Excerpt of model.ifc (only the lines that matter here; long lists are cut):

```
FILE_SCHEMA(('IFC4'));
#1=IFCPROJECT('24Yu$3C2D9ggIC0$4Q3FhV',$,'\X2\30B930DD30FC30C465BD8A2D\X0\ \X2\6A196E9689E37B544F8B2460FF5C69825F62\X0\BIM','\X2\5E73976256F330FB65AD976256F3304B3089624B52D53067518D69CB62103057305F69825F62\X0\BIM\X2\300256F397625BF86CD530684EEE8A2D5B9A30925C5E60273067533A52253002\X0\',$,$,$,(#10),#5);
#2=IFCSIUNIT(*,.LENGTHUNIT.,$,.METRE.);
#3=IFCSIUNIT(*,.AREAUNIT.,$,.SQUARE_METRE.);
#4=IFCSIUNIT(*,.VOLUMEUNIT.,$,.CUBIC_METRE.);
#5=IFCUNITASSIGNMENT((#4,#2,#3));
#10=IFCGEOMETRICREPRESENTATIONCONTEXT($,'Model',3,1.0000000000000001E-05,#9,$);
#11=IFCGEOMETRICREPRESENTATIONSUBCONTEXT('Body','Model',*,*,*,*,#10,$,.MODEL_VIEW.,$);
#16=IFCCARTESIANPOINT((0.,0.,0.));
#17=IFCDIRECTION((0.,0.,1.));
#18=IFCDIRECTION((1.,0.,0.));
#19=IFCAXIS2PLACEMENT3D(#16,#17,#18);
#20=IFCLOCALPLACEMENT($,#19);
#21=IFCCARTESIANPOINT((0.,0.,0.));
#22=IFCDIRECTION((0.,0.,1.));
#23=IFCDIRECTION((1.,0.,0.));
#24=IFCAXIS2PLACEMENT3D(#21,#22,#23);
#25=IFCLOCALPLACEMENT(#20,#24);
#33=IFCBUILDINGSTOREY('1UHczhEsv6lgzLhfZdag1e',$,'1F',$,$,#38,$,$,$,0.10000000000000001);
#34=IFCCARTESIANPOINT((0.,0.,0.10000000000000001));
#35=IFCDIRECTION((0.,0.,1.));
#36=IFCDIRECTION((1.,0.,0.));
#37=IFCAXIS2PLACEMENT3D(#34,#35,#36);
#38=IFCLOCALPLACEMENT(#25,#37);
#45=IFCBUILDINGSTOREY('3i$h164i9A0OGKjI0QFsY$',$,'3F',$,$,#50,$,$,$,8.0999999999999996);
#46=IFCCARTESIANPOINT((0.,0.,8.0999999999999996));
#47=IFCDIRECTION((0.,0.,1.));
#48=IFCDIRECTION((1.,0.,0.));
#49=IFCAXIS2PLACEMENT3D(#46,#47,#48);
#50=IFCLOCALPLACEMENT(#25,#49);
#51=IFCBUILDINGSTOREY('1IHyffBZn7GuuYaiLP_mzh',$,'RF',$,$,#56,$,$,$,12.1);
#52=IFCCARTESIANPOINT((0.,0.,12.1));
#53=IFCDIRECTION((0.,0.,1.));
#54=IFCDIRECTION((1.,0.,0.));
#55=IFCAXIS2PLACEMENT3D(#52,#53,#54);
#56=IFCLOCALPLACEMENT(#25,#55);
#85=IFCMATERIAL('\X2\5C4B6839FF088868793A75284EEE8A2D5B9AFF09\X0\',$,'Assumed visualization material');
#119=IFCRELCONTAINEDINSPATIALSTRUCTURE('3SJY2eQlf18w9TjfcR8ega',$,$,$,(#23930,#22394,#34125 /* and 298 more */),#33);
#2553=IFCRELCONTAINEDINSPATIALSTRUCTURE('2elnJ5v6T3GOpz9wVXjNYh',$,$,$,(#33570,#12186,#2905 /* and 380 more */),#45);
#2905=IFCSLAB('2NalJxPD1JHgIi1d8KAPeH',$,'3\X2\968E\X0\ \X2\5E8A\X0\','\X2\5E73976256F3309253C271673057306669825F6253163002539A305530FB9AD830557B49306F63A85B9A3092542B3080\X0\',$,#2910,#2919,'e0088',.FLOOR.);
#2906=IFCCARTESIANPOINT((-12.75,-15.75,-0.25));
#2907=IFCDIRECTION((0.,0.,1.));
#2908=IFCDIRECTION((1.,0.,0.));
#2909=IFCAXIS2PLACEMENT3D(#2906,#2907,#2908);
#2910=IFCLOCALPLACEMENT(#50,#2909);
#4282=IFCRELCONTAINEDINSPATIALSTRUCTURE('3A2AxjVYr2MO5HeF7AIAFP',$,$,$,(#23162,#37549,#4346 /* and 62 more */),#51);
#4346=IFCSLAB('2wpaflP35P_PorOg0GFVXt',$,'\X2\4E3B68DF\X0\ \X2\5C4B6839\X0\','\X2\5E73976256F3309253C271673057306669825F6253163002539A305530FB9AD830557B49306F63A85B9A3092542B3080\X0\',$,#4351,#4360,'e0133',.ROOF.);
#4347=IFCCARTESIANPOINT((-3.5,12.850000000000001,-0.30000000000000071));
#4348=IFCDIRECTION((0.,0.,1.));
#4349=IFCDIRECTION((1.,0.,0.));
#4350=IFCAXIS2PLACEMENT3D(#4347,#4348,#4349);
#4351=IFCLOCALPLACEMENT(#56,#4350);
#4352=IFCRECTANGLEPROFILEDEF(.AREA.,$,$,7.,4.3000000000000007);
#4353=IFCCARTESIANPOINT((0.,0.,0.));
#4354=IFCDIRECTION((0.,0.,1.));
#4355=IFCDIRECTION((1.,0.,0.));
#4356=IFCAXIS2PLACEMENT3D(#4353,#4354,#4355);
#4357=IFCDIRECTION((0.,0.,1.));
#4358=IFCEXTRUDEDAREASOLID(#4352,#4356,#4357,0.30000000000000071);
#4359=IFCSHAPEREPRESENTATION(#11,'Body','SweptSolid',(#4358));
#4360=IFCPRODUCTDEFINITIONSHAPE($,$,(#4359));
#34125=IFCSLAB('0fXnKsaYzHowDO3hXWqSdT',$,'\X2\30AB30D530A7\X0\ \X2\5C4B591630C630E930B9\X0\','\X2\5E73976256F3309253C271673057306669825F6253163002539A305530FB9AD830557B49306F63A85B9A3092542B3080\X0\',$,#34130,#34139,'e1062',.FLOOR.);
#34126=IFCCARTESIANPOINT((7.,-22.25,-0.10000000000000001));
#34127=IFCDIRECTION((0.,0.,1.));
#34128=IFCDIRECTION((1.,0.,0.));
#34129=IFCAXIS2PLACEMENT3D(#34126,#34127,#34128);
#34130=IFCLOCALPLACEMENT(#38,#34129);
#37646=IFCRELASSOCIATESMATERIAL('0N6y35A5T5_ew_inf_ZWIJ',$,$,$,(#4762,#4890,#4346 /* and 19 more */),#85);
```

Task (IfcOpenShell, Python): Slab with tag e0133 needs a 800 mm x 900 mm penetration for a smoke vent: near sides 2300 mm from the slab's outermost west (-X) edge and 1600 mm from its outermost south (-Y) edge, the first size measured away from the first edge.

```python
import numpy as np
import ifcopenshell
import ifcopenshell.api.feature
import ifcopenshell.api.geometry
import ifcopenshell.api.root
import ifcopenshell.geom
import ifcopenshell.util.placement
import ifcopenshell.util.representation
import ifcopenshell.util.shape
import ifcopenshell.util.unit

model = ifcopenshell.open("model.ifc")
unit_scale = ifcopenshell.util.unit.calculate_unit_scale(model)
settings = ifcopenshell.geom.settings()


def volume(element):
    """Net volume in cubic metres, openings subtracted."""
    shape = ifcopenshell.geom.create_shape(settings, element)
    return ifcopenshell.util.shape.get_volume(shape.geometry)


slab = model.by_guid("2wpaflP35P_PorOg0GFVXt")
before = volume(slab)

# Extent in the slab's own axes, in metres. The edges named are its -X and -Y sides.
slab_shape = ifcopenshell.geom.create_shape(settings, slab)
vertices = ifcopenshell.util.shape.get_vertices(slab_shape.geometry)
x_min, y_min, bottom = vertices.min(axis=0)
top = vertices[:, 2].max()

opening = ifcopenshell.api.root.create_entity(model, ifc_class="IfcOpeningElement", name="Smoke vent opening", predefined_type="OPENING")
context = ifcopenshell.util.representation.get_context(model, "Model", "Body", "MODEL_VIEW")
width, depth = 0.8, 0.9
outline = [(0.0, 0.0), (width, 0.0), (width, depth), (0.0, depth), (0.0, 0.0)]
# Overshoot both faces by 50 mm so the cut is clean.
shape = ifcopenshell.api.geometry.add_slab_representation(
    model, context=context, depth=top - bottom + 0.1, polyline=outline
)
ifcopenshell.api.geometry.assign_representation(model, product=opening, representation=shape)

matrix = ifcopenshell.util.placement.get_local_placement(slab.ObjectPlacement)
matrix[:, 3] = matrix @ np.append(np.array([x_min + 2.3, y_min + 1.6, bottom - 0.05]) / unit_scale, 1.0)
ifcopenshell.api.geometry.edit_object_placement(model, product=opening, matrix=matrix, is_si=False)
ifcopenshell.api.feature.add_feature(model, feature=opening, element=slab)

after = volume(slab)

print(f"slab volume {before:.3f} -> {after:.3f} m3")

model.write("model_edited.ifc")
```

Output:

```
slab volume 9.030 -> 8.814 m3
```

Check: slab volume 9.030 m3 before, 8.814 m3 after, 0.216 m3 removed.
